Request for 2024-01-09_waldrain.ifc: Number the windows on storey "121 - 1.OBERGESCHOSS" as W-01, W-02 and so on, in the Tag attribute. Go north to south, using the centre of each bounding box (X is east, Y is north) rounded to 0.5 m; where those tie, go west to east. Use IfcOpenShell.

First a look at what the model holds.

```python
import ifcopenshell
import ifcopenshell.util.element
import ifcopenshell.util.placement

model = ifcopenshell.open("2024-01-09_waldrain.ifc")
print(model.schema)
storey = next(s for s in model.by_type("IfcBuildingStorey") if s.Name == "121 - 1.OBERGESCHOSS")
windows = [e for e in ifcopenshell.util.element.get_decomposition(storey) if e.is_a("IfcWindow")]
for e in sorted(windows, key=lambda e: e.id()):
    origin = ifcopenshell.util.placement.get_local_placement(e.ObjectPlacement)[:3, 3]
    print(e.id(), e.Tag, e.Name, origin.round(2) + 0.0, sep=" | ")
```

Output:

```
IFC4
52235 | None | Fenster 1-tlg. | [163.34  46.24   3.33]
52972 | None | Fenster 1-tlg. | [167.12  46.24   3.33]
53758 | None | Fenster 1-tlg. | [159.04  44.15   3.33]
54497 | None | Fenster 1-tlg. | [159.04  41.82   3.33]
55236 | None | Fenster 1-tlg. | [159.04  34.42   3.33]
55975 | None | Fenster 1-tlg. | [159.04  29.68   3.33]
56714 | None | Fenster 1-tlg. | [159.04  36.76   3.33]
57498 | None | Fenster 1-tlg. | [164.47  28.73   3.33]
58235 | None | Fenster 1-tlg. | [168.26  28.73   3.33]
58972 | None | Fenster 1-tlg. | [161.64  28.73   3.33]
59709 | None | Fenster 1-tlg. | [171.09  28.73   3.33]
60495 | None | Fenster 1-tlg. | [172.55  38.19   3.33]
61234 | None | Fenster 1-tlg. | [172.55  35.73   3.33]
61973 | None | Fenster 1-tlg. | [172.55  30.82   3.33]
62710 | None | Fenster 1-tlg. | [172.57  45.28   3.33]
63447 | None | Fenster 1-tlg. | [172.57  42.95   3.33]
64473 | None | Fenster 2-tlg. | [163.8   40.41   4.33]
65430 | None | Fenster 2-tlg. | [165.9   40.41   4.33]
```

```python
import ifcopenshell
import ifcopenshell.geom
import ifcopenshell.util.element
import ifcopenshell.util.shape

model = ifcopenshell.open("2024-01-09_waldrain.ifc")
settings = ifcopenshell.geom.settings()
settings.set("use-world-coords", True)


def centre(element):
    shape = ifcopenshell.geom.create_shape(settings, element)
    return ifcopenshell.util.shape.get_bbox_centroid(shape.geometry)


storey = next(s for s in model.by_type("IfcBuildingStorey") if s.Name == "121 - 1.OBERGESCHOSS")
windows = [e for e in ifcopenshell.util.element.get_decomposition(storey) if e.is_a("IfcWindow")]

# Insertion points can sit at a corner or the storey origin, so sort by the geometry (in metres).
centres = {e: centre(e) for e in windows}
windows.sort(key=lambda e: (-round(centres[e][1] / 0.5), centres[e][0]))

for i, e in enumerate(windows, start=1):
    number = f"W-{i:02d}"
    e.Tag = number
    print(e.id(), number)

model.write("2024-01-09_waldrain_v2.ifc")
```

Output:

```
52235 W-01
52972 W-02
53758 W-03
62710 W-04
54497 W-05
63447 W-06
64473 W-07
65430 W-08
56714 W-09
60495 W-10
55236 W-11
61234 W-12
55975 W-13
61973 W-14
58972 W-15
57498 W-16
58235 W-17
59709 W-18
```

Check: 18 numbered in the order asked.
